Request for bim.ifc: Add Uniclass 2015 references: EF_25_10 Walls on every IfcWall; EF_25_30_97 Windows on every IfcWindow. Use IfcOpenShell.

First a look at what the model holds.

```python
import ifcopenshell

model = ifcopenshell.open("bim.ifc")
print(model.schema)
print("classifications:", [c.Name for c in model.by_type("IfcClassification")])
for ifc_class in ("IfcDoor", "IfcRoof", "IfcStair", "IfcWall", "IfcWindow"):
    print(ifc_class, len(model.by_type(ifc_class)))
```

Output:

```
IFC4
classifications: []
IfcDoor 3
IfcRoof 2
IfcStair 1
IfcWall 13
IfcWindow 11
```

```python
import ifcopenshell
import ifcopenshell.api.classification

model = ifcopenshell.open("bim.ifc")

system = ifcopenshell.api.classification.add_classification(model, classification="Uniclass 2015")

codes = {
    "IfcWall": ("EF_25_10", "Walls"),
    "IfcWindow": ("EF_25_30_97", "Windows"),
}
for ifc_class, (code, name) in codes.items():
    products = model.by_type(ifc_class)
    ifcopenshell.api.classification.add_reference(
        model, products=products, classification=system, identification=code, name=name
    )
    print(code, len(products))

model.write("bim_edited.ifc")
```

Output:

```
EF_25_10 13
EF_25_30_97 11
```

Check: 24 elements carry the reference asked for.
